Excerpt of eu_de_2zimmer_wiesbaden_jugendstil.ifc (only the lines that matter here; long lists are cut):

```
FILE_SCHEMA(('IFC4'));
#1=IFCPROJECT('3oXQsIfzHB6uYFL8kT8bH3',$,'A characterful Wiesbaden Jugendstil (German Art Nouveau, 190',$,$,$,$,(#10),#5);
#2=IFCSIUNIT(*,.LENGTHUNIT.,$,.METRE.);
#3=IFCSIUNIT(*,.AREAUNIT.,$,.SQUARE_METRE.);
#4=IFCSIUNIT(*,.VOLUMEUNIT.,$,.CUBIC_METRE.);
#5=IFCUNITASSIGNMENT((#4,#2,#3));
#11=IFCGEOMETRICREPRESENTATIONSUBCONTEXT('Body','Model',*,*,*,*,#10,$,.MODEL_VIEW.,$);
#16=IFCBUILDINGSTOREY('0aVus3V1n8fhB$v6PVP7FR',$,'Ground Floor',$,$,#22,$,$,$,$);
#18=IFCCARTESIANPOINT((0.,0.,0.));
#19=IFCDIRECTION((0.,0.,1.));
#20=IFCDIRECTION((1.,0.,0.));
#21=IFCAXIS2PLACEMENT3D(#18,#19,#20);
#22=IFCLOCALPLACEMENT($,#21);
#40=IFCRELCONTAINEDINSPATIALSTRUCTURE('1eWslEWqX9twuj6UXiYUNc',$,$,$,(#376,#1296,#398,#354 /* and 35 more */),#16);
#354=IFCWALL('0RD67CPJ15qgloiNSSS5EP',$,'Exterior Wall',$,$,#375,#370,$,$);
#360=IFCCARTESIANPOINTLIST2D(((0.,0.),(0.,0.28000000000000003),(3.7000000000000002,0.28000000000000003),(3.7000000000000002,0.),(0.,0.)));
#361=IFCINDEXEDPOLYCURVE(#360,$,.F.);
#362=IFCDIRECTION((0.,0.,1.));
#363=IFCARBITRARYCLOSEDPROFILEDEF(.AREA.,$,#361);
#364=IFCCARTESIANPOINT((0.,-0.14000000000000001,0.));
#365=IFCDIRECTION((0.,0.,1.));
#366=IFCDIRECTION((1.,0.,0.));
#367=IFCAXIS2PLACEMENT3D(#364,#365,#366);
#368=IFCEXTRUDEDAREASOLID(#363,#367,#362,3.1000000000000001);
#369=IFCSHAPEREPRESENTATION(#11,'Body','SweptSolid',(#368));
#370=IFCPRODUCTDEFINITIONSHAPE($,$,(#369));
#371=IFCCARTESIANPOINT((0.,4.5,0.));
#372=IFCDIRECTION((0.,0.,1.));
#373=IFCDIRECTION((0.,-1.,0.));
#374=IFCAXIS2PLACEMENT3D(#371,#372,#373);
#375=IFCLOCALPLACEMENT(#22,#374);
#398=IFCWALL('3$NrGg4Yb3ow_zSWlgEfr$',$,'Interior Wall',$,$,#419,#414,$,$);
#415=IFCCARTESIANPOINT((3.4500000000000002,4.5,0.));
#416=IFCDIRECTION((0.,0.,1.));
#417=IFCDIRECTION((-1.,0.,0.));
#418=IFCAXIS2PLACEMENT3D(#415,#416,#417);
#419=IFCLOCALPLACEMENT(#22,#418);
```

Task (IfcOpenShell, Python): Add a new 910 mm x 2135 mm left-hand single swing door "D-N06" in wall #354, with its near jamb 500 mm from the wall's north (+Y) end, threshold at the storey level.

```python
import numpy as np
import ifcopenshell
import ifcopenshell.api.feature
import ifcopenshell.api.geometry
import ifcopenshell.api.root
import ifcopenshell.api.spatial
import ifcopenshell.geom
import ifcopenshell.util.element
import ifcopenshell.util.placement
import ifcopenshell.util.representation
import ifcopenshell.util.shape
import ifcopenshell.util.unit

model = ifcopenshell.open("eu_de_2zimmer_wiesbaden_jugendstil.ifc")
unit_scale = ifcopenshell.util.unit.calculate_unit_scale(model)
settings = ifcopenshell.geom.settings()


def volume(element):
    """Net volume in cubic metres, openings subtracted."""
    shape = ifcopenshell.geom.create_shape(settings, element)
    return ifcopenshell.util.shape.get_volume(shape.geometry)


wall = model.by_guid("0RD67CPJ15qgloiNSSS5EP")
storey = ifcopenshell.util.element.get_container(wall, ifc_class="IfcBuildingStorey")
context = ifcopenshell.util.representation.get_context(model, "Model", "Body", "MODEL_VIEW")
before = volume(wall)

width, height, from_end, sill = 0.91, 2.135, 0.5, 0.0  # metres

# The wall runs along its own X axis, and the end named is its -X end.
wall_shape = ifcopenshell.geom.create_shape(settings, wall)
x, y, z = ifcopenshell.util.shape.get_vertices(wall_shape.geometry).T
start = x.min() + from_end
face, thickness = float(y.min()), float(y.max() - y.min())
wall_matrix = ifcopenshell.util.placement.get_local_placement(wall.ObjectPlacement)
level = ifcopenshell.util.placement.get_local_placement(storey.ObjectPlacement)[2, 3]


def in_wall(x, y):
    """Placement at x, y metres in the wall's axes, at sill height."""
    matrix = wall_matrix.copy()
    matrix[:, 3] = wall_matrix @ np.array([x / unit_scale, y / unit_scale, 0.0, 1.0])
    matrix[2, 3] = level + sill / unit_scale
    return matrix


# Opening: a box that overshoots both wall faces by 50 mm.
opening = ifcopenshell.api.root.create_entity(model, ifc_class="IfcOpeningElement", predefined_type="OPENING")
box = ifcopenshell.api.geometry.add_wall_representation(
    model, context=context, length=width, height=height, thickness=thickness + 0.1
)
ifcopenshell.api.geometry.assign_representation(model, product=opening, representation=box)
ifcopenshell.api.geometry.edit_object_placement(model, product=opening, matrix=in_wall(start, face - 0.05), is_si=False)
ifcopenshell.api.feature.add_feature(model, feature=opening, element=wall)

door = ifcopenshell.api.root.create_entity(model, ifc_class="IfcDoor", name="D-N06", predefined_type="DOOR")
door.OverallWidth, door.OverallHeight = width / unit_scale, height / unit_scale
door.OperationType = "SINGLE_SWING_LEFT"
body = ifcopenshell.api.geometry.add_door_representation(
    model,
    context=context,
    overall_width=door.OverallWidth,
    overall_height=door.OverallHeight,
    operation_type="SINGLE_SWING_LEFT",
    lining_properties={"LiningDepth": thickness / unit_scale, "ThresholdDepth": thickness / unit_scale},
)
ifcopenshell.api.geometry.assign_representation(model, product=door, representation=body)
ifcopenshell.api.spatial.assign_container(model, products=[door], relating_structure=storey)
ifcopenshell.api.feature.add_filling(model, opening=opening, element=door)

# The lining spans the wall, so the door starts at the wall face.
ifcopenshell.api.geometry.edit_object_placement(model, product=door, matrix=in_wall(start, face), is_si=False)

after = volume(wall)

print(f"wall volume {before:.3f} -> {after:.3f} m3")

model.write("eu_de_2zimmer_wiesbaden_jugendstil-out.ifc")
```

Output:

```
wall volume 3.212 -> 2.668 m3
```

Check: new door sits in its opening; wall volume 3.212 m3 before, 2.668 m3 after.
